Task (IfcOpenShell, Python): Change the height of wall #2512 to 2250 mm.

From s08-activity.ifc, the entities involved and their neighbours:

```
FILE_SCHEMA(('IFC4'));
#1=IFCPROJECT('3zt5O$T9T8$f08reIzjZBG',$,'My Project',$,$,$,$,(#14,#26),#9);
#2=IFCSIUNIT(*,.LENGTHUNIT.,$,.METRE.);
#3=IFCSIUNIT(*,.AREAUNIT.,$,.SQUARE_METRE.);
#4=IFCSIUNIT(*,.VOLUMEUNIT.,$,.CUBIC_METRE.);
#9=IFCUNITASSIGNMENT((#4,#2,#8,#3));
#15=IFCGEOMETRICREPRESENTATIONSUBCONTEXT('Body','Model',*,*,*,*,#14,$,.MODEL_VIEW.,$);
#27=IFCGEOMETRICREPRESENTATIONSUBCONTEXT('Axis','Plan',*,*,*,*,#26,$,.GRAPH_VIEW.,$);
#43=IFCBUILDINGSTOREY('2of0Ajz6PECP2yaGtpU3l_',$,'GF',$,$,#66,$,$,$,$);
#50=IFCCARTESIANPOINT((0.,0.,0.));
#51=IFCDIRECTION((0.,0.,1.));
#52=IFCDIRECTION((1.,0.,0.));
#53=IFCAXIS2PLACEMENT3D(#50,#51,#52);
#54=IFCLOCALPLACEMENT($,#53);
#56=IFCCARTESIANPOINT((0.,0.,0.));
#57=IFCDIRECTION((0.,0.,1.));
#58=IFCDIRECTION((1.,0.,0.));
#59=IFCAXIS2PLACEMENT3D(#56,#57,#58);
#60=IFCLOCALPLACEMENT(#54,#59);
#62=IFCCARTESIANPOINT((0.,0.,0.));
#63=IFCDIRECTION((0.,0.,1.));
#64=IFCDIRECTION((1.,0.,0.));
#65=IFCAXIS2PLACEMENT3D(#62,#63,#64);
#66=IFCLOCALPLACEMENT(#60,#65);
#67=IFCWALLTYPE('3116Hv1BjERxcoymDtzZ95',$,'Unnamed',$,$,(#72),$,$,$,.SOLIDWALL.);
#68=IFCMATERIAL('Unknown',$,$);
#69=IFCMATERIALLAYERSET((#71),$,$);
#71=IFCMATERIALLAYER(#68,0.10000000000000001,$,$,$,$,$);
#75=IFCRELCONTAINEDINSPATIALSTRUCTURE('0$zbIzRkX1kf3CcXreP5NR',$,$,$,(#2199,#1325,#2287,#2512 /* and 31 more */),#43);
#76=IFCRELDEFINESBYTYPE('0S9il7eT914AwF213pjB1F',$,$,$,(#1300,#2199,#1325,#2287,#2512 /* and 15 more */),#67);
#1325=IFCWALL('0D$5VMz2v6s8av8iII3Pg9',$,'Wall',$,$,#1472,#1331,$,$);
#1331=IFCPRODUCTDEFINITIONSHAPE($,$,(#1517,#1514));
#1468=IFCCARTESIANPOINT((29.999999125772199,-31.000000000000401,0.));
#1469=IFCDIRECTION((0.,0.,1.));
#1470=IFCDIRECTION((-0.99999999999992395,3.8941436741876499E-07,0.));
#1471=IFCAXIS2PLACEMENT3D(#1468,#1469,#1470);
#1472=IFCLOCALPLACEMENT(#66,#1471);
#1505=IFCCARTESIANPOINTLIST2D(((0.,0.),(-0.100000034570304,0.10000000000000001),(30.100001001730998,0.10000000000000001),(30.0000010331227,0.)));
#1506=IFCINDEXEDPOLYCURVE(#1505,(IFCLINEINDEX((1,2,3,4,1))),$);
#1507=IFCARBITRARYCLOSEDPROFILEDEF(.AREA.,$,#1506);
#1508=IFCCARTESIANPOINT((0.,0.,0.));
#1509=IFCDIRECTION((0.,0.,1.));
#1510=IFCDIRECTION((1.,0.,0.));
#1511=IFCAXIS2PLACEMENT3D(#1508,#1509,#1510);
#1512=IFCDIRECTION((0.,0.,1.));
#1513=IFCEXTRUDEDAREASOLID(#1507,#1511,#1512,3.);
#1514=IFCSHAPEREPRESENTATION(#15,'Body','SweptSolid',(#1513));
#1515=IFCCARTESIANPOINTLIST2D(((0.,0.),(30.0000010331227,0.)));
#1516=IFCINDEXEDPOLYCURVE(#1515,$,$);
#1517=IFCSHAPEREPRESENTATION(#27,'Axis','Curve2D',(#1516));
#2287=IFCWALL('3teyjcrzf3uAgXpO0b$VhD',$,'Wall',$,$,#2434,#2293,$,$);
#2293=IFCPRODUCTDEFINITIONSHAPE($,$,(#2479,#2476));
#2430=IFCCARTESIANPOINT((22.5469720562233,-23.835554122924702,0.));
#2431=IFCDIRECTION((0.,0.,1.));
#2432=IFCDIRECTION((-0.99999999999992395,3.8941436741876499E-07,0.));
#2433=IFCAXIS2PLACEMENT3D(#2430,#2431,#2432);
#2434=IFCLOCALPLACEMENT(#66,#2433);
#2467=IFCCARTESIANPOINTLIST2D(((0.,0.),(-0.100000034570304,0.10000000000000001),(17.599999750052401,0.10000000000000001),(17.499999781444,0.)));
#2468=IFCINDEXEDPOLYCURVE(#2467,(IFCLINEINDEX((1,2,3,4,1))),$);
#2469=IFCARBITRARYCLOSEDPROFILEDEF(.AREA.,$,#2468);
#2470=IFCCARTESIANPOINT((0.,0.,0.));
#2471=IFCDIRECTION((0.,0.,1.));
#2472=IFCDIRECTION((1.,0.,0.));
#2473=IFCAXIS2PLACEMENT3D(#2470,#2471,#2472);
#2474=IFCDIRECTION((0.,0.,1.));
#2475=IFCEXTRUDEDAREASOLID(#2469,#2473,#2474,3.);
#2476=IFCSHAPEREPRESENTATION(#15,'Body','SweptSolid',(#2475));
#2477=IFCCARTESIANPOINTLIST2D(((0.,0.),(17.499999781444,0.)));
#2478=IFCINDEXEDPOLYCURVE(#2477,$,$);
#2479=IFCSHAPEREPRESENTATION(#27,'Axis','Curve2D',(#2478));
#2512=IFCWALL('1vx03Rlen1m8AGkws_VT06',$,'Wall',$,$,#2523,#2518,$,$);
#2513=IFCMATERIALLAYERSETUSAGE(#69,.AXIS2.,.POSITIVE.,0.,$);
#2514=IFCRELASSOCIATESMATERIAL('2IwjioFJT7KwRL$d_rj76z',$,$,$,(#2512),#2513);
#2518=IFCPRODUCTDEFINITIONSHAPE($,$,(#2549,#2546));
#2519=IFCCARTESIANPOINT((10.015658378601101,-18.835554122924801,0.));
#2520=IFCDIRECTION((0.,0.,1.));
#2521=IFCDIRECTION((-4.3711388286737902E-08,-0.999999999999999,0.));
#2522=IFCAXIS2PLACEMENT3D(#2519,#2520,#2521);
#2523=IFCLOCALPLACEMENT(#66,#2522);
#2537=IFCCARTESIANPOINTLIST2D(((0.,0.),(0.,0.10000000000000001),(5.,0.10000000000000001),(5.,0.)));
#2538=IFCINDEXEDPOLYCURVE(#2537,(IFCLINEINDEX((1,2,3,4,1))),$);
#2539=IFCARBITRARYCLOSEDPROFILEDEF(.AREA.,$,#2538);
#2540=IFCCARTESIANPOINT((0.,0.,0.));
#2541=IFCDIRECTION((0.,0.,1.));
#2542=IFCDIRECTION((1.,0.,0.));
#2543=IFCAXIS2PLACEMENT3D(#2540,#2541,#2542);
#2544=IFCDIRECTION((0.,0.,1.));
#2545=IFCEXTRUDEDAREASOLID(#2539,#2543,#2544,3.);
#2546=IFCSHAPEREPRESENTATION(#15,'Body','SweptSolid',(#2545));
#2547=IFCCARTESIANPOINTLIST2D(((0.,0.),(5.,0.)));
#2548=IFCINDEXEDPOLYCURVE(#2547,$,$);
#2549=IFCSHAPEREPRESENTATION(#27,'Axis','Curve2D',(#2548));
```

```python
import ifcopenshell
import ifcopenshell.geom
import ifcopenshell.util.representation
import ifcopenshell.util.shape
import ifcopenshell.util.unit

model = ifcopenshell.open("s08-activity.ifc")
unit_scale = ifcopenshell.util.unit.calculate_unit_scale(model)
settings = ifcopenshell.geom.settings()


def volume(element):
    """Net volume in cubic metres, openings subtracted."""
    shape = ifcopenshell.geom.create_shape(settings, element)
    return ifcopenshell.util.shape.get_volume(shape.geometry)


wall = model.by_guid("1vx03Rlen1m8AGkws_VT06")
before = volume(wall)

body = ifcopenshell.util.representation.get_representation(wall, "Model", "Body")
solid = body.Items[0]
old_height = solid.Depth
solid.Depth = 2.25 / unit_scale
after = volume(wall)

print(f"height {old_height:g} -> {solid.Depth:g}, volume {before:.3f} -> {after:.3f} m3")

model.write("s08-activity-out.ifc")
```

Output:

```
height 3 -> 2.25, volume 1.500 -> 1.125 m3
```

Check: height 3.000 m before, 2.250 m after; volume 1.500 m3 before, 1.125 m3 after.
